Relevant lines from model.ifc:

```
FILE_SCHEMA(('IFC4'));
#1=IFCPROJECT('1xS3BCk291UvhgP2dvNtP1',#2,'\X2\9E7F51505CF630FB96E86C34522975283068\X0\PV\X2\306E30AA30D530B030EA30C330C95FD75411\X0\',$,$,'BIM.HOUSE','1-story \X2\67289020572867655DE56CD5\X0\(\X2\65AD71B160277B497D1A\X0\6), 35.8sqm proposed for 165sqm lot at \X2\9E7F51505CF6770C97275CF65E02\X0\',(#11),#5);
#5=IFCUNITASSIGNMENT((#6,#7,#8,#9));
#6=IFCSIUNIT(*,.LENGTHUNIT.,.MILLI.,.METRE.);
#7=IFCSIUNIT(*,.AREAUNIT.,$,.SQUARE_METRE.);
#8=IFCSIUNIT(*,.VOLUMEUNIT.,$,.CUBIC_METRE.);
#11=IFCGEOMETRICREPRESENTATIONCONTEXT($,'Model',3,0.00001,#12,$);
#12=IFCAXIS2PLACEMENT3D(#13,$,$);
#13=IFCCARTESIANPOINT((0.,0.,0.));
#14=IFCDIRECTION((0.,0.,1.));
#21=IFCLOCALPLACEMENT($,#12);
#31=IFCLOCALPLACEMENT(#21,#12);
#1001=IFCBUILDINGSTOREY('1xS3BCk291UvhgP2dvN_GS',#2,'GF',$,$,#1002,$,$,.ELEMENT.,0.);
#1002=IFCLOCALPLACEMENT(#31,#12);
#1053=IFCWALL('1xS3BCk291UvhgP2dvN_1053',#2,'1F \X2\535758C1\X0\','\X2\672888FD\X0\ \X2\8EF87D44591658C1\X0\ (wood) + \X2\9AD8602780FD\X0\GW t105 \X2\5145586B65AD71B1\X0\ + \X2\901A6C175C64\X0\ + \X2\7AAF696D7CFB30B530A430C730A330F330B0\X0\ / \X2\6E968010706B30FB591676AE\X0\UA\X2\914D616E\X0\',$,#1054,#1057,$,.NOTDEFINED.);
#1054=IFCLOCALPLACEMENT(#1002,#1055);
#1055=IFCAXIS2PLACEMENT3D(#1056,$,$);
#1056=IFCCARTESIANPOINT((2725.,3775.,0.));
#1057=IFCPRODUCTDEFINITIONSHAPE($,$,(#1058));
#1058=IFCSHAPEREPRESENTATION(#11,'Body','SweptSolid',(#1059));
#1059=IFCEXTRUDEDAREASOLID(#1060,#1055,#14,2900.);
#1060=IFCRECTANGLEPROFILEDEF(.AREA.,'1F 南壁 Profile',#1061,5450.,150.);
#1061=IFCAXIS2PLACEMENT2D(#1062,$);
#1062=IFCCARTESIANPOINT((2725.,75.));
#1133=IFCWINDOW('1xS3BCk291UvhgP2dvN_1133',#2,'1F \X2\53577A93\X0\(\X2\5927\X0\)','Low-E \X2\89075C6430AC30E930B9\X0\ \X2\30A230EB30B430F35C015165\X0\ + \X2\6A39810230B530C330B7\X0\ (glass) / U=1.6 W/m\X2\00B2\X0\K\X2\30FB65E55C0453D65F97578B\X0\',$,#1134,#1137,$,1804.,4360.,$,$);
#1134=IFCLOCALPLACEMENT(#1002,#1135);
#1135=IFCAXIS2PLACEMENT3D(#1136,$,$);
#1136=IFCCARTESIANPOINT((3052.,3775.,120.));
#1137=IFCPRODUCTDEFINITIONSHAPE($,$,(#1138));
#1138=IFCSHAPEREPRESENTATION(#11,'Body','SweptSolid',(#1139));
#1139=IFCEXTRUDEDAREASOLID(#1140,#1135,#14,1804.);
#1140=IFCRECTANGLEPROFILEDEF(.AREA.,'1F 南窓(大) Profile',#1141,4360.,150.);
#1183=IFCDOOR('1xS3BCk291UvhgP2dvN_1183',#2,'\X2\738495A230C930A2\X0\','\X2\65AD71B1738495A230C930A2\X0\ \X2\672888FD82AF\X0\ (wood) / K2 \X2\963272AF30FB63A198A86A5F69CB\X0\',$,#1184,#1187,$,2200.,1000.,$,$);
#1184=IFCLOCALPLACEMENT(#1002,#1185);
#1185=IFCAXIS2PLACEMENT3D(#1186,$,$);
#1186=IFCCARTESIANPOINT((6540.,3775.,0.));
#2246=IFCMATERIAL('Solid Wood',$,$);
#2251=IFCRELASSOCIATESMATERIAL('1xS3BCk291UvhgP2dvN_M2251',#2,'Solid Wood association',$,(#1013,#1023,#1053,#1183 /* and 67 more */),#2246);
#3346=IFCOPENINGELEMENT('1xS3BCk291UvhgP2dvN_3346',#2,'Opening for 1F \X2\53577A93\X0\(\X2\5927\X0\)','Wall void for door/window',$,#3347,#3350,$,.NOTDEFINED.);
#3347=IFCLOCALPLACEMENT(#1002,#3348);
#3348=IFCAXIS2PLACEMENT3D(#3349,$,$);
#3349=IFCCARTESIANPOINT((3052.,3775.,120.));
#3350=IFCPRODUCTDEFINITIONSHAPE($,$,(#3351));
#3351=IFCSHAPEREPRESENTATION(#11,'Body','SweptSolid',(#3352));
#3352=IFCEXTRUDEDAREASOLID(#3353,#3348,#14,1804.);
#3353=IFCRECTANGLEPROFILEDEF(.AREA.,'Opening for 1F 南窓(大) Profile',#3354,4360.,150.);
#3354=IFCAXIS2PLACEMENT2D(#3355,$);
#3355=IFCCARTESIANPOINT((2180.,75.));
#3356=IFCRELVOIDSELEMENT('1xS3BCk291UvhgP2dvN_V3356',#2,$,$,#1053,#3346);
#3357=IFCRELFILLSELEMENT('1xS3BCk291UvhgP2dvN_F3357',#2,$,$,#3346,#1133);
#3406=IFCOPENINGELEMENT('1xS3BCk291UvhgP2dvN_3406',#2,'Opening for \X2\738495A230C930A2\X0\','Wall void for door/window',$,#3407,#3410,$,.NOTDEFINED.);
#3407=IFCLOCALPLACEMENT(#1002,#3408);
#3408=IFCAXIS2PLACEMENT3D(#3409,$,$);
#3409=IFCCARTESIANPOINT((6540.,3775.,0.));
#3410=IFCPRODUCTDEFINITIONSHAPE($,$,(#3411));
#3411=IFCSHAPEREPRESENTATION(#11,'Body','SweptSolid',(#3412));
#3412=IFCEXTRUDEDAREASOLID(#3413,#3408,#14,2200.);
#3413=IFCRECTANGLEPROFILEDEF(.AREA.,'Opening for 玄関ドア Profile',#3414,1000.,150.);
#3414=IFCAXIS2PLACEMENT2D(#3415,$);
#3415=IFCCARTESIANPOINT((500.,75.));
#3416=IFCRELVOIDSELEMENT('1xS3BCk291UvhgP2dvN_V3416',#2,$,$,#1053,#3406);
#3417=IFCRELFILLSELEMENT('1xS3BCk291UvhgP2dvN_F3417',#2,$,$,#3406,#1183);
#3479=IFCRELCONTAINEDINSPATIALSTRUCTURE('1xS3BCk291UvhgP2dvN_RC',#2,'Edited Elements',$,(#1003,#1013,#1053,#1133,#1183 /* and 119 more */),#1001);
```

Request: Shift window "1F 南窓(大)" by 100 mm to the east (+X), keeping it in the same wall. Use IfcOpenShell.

```python
import ifcopenshell
import ifcopenshell.api.geometry
import ifcopenshell.util.placement

model = ifcopenshell.open("model.ifc")

window = model.by_guid("1xS3BCk291UvhgP2dvN_1133")
opening = window.FillsVoids[0].RelatingOpeningElement
wall = opening.VoidsElements[0].RelatingBuildingElement

wall_matrix = ifcopenshell.util.placement.get_local_placement(wall.ObjectPlacement)
shift = wall_matrix[:3, 0] * 100.0
before = ifcopenshell.util.placement.get_local_placement(window.ObjectPlacement)[:3, 3].copy()

# The window is not placed relative to its opening, so move both.
for product in (opening, window):
    matrix = ifcopenshell.util.placement.get_local_placement(product.ObjectPlacement)
    matrix[:3, 3] += shift
    ifcopenshell.api.geometry.edit_object_placement(model, product=product, matrix=matrix, is_si=False)

after = ifcopenshell.util.placement.get_local_placement(window.ObjectPlacement)[:3, 3]
print("window moved by", (after - before).round(3) + 0.0)

model.write("model_rev.ifc")
```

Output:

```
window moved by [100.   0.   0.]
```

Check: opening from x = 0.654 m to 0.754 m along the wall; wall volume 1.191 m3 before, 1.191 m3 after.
